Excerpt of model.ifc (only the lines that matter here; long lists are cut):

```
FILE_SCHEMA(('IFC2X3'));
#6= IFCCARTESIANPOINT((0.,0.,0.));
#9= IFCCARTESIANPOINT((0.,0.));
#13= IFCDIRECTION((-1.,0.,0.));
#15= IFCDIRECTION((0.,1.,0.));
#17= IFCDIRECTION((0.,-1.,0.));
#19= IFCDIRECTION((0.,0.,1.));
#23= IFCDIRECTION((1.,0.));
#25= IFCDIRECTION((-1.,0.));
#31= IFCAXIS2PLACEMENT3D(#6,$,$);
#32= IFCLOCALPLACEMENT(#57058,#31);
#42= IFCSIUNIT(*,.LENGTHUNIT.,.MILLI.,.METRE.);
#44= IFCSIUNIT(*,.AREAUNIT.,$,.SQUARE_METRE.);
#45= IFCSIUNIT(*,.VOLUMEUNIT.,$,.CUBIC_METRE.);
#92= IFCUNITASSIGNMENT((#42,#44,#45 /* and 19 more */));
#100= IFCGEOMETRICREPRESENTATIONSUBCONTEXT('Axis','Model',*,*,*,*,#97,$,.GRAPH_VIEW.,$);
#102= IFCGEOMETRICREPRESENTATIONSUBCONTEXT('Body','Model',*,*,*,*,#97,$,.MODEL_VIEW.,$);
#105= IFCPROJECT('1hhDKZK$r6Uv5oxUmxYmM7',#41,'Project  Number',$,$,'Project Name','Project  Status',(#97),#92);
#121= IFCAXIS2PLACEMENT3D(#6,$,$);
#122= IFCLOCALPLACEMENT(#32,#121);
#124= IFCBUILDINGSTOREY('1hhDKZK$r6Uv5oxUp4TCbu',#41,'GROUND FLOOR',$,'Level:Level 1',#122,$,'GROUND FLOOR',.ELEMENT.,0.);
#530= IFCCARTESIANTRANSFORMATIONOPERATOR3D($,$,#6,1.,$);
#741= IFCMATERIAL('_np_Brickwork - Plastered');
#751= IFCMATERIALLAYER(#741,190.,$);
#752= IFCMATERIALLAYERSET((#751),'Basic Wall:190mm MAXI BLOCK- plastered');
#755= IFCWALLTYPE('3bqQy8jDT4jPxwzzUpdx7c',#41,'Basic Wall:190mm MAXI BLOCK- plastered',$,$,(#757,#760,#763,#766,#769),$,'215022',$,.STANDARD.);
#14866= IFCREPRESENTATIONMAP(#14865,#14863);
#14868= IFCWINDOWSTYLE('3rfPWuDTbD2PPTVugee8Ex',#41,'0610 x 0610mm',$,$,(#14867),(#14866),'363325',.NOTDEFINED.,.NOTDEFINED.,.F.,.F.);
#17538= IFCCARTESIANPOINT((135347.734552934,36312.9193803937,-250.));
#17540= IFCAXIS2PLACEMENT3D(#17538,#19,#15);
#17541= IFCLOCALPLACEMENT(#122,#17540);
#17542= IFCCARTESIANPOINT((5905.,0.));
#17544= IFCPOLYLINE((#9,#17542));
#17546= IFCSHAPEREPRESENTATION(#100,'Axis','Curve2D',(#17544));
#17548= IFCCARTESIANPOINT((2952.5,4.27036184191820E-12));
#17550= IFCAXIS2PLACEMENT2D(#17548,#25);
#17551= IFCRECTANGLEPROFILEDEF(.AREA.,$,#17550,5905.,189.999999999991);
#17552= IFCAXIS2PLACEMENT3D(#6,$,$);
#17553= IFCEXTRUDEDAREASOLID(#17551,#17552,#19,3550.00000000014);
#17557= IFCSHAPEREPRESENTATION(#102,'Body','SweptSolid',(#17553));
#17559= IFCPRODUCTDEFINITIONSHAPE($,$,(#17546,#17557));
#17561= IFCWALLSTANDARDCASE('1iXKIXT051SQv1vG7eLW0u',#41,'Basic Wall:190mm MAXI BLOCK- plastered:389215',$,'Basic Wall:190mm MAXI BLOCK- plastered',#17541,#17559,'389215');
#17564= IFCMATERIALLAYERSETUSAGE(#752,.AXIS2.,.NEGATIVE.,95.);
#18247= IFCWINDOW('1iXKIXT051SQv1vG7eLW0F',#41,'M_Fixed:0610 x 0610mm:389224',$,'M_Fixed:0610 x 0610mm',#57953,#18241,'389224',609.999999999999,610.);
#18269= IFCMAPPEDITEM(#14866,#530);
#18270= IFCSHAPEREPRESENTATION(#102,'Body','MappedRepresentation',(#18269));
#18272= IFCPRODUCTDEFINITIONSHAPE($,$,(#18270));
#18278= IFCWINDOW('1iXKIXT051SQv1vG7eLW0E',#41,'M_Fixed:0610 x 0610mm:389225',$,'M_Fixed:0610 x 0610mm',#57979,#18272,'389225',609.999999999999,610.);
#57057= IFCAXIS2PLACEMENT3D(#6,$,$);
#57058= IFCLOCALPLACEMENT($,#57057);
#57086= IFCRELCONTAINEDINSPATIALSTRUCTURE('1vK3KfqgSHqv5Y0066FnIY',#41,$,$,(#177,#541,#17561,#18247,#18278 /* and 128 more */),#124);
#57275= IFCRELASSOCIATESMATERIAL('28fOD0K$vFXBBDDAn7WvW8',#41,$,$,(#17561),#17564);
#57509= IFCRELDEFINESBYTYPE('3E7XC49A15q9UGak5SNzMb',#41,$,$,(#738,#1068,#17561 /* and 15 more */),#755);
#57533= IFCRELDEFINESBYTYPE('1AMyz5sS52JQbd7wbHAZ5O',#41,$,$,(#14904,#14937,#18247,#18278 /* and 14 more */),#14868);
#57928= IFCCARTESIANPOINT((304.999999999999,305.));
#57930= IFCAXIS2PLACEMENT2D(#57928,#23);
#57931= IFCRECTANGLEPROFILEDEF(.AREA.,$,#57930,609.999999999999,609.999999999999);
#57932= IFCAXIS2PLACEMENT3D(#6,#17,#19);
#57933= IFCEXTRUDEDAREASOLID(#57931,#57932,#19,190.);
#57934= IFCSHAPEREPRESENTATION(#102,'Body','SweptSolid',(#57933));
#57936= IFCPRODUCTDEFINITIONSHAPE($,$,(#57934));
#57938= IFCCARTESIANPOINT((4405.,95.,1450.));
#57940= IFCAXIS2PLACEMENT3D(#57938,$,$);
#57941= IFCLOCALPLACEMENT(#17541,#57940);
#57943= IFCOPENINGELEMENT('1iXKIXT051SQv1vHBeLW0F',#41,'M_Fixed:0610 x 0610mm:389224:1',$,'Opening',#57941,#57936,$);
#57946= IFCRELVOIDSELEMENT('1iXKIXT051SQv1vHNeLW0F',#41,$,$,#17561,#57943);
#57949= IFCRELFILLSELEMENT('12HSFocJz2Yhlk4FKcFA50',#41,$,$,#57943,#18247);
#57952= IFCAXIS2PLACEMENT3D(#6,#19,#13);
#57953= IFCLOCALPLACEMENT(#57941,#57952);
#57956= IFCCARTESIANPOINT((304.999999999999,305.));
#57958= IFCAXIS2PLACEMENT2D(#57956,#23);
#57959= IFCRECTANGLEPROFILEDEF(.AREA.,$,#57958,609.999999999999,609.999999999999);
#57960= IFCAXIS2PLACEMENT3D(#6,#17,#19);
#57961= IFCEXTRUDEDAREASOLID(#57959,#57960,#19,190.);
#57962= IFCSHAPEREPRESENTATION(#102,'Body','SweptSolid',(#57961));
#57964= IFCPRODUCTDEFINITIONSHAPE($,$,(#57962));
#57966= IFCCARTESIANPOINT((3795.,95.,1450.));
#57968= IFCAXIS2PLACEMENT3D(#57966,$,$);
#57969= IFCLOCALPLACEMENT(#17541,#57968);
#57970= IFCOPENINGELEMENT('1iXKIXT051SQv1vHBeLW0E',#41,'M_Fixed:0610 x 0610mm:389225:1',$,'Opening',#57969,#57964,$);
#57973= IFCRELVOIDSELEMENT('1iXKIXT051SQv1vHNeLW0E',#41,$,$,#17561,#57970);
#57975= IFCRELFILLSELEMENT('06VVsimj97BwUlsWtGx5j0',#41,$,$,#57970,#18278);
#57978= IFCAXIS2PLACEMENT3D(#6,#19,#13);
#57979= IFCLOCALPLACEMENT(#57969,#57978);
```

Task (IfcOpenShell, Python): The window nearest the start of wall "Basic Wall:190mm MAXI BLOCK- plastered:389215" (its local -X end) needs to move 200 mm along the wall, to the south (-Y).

```python
import ifcopenshell
import ifcopenshell.api.geometry
import ifcopenshell.util.placement

model = ifcopenshell.open("model.ifc")

window = model.by_id(18278)
opening = window.FillsVoids[0].RelatingOpeningElement
wall = opening.VoidsElements[0].RelatingBuildingElement

wall_matrix = ifcopenshell.util.placement.get_local_placement(wall.ObjectPlacement)
shift = wall_matrix[:3, 0] * -200.0
before = ifcopenshell.util.placement.get_local_placement(window.ObjectPlacement)[:3, 3].copy()

# The window is placed relative to its opening, so it follows when the opening moves.
matrix = ifcopenshell.util.placement.get_local_placement(opening.ObjectPlacement)
matrix[:3, 3] += shift
ifcopenshell.api.geometry.edit_object_placement(
    model, product=opening, matrix=matrix, is_si=False, should_transform_children=True
)

after = ifcopenshell.util.placement.get_local_placement(window.ObjectPlacement)[:3, 3]
print("window moved by", (after - before).round(3) + 0.0)

model.write("model_rev.ifc")
```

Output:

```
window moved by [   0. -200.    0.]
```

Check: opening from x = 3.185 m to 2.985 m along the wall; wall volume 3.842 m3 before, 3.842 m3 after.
